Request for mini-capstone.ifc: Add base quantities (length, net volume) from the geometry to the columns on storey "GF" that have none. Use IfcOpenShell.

First a look at what the model holds.

```python
import ifcopenshell
import ifcopenshell.util.element
import ifcopenshell.util.unit

model = ifcopenshell.open("mini-capstone.ifc")
print(model.schema)
for unit_type in ("LENGTHUNIT", "AREAUNIT", "VOLUMEUNIT"):
    print(unit_type, ifcopenshell.util.unit.calculate_unit_scale(model, unit_type))
storey = next(s for s in model.by_type("IfcBuildingStorey") if s.Name == "GF")
columns = [e for e in ifcopenshell.util.element.get_decomposition(storey) if e.is_a("IfcColumn")]
for e in sorted(columns, key=lambda e: e.id()):
    print(e.id(), e.is_a(), e.Name, list(ifcopenshell.util.element.get_psets(e, qtos_only=True)), sep=" | ")
```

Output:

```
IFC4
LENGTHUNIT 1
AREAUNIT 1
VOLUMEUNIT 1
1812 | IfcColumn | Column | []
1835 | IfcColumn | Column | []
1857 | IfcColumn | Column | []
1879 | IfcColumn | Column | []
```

```python
import ifcopenshell
import ifcopenshell.api.pset
import ifcopenshell.geom
import ifcopenshell.util.element
import ifcopenshell.util.shape
import ifcopenshell.util.unit

model = ifcopenshell.open("mini-capstone.ifc")
unit_scale = ifcopenshell.util.unit.calculate_unit_scale(model)
volume_scale = ifcopenshell.util.unit.calculate_unit_scale(model, "VOLUMEUNIT")
settings = ifcopenshell.geom.settings()

storey = next(s for s in model.by_type("IfcBuildingStorey") if s.Name == "GF")
columns = [e for e in ifcopenshell.util.element.get_decomposition(storey) if e.is_a("IfcColumn")]

for e in sorted(columns, key=lambda e: e.id()):
    if ifcopenshell.util.element.get_psets(e, qtos_only=True, should_inherit=False):
        continue
    # Geometry comes back in metres, in the element's own axes.
    shape = ifcopenshell.geom.create_shape(settings, e)
    values = {
        "Length": ifcopenshell.util.shape.get_z(shape.geometry) / unit_scale,
        "NetVolume": ifcopenshell.util.shape.get_volume(shape.geometry) / volume_scale,
    }
    qto = ifcopenshell.api.pset.add_qto(model, product=e, name="Qto_ColumnBaseQuantities")
    ifcopenshell.api.pset.edit_qto(model, qto=qto, properties=values)
    print(e.id(), {k: round(v, 3) for k, v in values.items()})

model.write("mini-capstone_rev.ifc")
```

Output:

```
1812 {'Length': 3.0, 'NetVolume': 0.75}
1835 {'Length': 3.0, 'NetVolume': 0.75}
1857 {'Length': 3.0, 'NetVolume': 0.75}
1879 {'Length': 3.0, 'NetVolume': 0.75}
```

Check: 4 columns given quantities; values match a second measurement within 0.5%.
